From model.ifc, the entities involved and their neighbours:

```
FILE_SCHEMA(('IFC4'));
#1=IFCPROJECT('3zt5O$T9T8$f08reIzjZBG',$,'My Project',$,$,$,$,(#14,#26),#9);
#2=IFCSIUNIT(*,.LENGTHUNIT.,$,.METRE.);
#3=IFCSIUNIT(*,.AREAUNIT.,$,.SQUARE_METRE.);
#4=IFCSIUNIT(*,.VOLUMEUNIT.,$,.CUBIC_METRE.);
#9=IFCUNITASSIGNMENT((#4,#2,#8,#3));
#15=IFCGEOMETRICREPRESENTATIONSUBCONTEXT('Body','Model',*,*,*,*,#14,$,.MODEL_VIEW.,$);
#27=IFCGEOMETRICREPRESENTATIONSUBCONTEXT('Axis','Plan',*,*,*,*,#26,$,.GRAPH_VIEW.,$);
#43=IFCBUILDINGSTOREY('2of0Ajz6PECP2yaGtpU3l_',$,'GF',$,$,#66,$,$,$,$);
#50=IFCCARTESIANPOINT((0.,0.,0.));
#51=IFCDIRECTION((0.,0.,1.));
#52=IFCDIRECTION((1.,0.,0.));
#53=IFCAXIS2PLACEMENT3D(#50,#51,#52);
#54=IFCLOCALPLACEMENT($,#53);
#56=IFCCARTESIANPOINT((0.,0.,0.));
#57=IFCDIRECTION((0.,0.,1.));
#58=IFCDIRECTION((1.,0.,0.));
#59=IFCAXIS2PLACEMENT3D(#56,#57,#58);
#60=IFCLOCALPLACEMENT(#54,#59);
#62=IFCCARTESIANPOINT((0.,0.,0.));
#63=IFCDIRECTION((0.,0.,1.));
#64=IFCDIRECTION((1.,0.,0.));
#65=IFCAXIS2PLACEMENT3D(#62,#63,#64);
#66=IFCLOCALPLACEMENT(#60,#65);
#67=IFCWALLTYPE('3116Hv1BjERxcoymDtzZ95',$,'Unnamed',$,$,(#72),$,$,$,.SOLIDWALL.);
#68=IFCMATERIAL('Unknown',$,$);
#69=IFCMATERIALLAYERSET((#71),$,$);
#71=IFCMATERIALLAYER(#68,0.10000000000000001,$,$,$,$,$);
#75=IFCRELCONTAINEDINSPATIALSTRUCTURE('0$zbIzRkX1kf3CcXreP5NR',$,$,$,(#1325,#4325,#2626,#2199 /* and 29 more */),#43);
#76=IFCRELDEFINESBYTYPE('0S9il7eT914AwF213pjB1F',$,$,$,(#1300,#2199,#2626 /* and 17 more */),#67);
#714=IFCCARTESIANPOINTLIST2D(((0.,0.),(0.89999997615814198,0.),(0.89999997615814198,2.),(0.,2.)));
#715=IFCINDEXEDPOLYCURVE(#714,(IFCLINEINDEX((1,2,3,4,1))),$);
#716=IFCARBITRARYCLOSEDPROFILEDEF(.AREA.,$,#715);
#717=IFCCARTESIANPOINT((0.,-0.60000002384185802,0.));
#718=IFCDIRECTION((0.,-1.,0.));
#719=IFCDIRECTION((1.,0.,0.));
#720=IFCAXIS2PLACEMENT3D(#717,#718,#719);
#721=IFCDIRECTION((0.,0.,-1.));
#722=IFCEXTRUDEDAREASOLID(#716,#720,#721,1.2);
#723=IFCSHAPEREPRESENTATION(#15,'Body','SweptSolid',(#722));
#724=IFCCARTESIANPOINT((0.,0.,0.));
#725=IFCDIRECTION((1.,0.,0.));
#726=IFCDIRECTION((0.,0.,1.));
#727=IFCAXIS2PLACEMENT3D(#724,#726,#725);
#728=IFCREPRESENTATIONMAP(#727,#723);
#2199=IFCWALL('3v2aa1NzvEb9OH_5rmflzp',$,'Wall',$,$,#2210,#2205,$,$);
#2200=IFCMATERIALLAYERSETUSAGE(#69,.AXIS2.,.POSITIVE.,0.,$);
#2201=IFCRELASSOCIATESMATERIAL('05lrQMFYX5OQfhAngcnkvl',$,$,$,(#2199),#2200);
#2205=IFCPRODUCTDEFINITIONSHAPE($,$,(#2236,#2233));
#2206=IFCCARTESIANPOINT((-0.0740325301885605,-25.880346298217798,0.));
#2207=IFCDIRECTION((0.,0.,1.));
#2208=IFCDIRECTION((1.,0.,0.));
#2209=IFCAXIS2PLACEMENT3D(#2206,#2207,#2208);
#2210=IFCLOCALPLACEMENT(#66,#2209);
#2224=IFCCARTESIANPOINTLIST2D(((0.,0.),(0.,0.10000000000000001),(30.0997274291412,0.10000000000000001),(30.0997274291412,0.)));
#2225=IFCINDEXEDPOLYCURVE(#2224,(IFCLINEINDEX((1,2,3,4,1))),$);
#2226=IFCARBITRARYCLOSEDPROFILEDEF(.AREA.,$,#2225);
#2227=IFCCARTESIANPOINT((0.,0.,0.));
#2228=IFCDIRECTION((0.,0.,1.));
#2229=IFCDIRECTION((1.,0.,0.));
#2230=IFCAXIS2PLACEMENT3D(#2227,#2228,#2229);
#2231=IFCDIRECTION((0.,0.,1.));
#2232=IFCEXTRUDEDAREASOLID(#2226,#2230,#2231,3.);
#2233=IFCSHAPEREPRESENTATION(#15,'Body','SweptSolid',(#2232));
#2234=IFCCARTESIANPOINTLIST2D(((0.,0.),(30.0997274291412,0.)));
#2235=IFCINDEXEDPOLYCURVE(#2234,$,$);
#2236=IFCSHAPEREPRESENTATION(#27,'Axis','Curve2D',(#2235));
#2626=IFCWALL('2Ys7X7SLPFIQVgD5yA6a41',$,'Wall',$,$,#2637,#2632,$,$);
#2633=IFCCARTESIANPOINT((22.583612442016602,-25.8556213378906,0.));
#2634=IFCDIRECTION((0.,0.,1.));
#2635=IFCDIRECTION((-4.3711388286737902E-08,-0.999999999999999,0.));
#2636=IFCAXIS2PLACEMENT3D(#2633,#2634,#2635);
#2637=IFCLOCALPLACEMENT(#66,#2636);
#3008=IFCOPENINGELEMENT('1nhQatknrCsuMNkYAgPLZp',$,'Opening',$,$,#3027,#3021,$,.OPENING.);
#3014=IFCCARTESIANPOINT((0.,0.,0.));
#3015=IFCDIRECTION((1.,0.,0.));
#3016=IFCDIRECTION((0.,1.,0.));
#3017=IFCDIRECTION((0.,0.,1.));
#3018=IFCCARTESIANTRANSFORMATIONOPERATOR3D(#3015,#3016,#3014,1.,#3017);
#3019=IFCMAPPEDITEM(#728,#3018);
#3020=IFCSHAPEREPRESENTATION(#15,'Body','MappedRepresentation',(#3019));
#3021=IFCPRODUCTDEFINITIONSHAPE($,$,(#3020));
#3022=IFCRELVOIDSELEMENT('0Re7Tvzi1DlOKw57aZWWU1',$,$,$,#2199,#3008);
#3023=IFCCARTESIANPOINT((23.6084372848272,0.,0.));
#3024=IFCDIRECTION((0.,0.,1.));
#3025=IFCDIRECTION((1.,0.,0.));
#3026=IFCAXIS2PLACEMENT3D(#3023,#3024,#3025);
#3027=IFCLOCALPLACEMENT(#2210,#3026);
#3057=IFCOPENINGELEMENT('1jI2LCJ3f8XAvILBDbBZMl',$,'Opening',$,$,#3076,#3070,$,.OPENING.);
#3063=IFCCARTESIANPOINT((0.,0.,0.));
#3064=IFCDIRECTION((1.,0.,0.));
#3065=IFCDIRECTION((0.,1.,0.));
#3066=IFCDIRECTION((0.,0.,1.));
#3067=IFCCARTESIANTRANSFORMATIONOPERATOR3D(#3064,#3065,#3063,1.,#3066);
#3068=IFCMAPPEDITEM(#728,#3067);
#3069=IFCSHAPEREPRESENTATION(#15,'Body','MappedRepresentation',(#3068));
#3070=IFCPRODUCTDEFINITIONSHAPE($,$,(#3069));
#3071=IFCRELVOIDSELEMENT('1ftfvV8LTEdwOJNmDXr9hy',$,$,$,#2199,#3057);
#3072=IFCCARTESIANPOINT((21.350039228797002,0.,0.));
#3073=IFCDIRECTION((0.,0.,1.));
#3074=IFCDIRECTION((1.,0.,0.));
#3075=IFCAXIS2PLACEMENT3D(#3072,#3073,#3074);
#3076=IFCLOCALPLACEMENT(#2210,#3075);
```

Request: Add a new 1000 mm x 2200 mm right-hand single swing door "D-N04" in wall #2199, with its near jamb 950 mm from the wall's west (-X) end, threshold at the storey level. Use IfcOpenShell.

```python
import numpy as np
import ifcopenshell
import ifcopenshell.api.feature
import ifcopenshell.api.geometry
import ifcopenshell.api.root
import ifcopenshell.api.spatial
import ifcopenshell.geom
import ifcopenshell.util.element
import ifcopenshell.util.placement
import ifcopenshell.util.representation
import ifcopenshell.util.shape
import ifcopenshell.util.unit

model = ifcopenshell.open("model.ifc")
unit_scale = ifcopenshell.util.unit.calculate_unit_scale(model)
settings = ifcopenshell.geom.settings()


def volume(element):
    """Net volume in cubic metres, openings subtracted."""
    shape = ifcopenshell.geom.create_shape(settings, element)
    return ifcopenshell.util.shape.get_volume(shape.geometry)


wall = model.by_guid("3v2aa1NzvEb9OH_5rmflzp")
storey = ifcopenshell.util.element.get_container(wall, ifc_class="IfcBuildingStorey")
context = ifcopenshell.util.representation.get_context(model, "Model", "Body", "MODEL_VIEW")
before = volume(wall)

width, height, from_end, sill = 1, 2.2, 0.95, 0.0  # metres

# The wall runs along its own X axis, and the end named is its -X end.
wall_shape = ifcopenshell.geom.create_shape(settings, wall)
x, y, z = ifcopenshell.util.shape.get_vertices(wall_shape.geometry).T
start = x.min() + from_end
face, thickness = float(y.min()), float(y.max() - y.min())
wall_matrix = ifcopenshell.util.placement.get_local_placement(wall.ObjectPlacement)
level = ifcopenshell.util.placement.get_local_placement(storey.ObjectPlacement)[2, 3]


def in_wall(x, y):
    """Placement at x, y metres in the wall's axes, at sill height."""
    matrix = wall_matrix.copy()
    matrix[:, 3] = wall_matrix @ np.array([x / unit_scale, y / unit_scale, 0.0, 1.0])
    matrix[2, 3] = level + sill / unit_scale
    return matrix


# Opening: a box that overshoots both wall faces by 50 mm.
opening = ifcopenshell.api.root.create_entity(model, ifc_class="IfcOpeningElement", predefined_type="OPENING")
box = ifcopenshell.api.geometry.add_wall_representation(
    model, context=context, length=width, height=height, thickness=thickness + 0.1
)
ifcopenshell.api.geometry.assign_representation(model, product=opening, representation=box)
ifcopenshell.api.geometry.edit_object_placement(model, product=opening, matrix=in_wall(start, face - 0.05), is_si=False)
ifcopenshell.api.feature.add_feature(model, feature=opening, element=wall)

door = ifcopenshell.api.root.create_entity(model, ifc_class="IfcDoor", name="D-N04", predefined_type="DOOR")
door.OverallWidth, door.OverallHeight = width / unit_scale, height / unit_scale
door.OperationType = "SINGLE_SWING_RIGHT"
body = ifcopenshell.api.geometry.add_door_representation(
    model,
    context=context,
    overall_width=door.OverallWidth,
    overall_height=door.OverallHeight,
    operation_type="SINGLE_SWING_RIGHT",
    lining_properties={"LiningDepth": thickness / unit_scale, "ThresholdDepth": thickness / unit_scale},
)
ifcopenshell.api.geometry.assign_representation(model, product=door, representation=body)
ifcopenshell.api.spatial.assign_container(model, products=[door], relating_structure=storey)
ifcopenshell.api.feature.add_filling(model, opening=opening, element=door)

# The lining spans the wall, so the door starts at the wall face.
ifcopenshell.api.geometry.edit_object_placement(model, product=door, matrix=in_wall(start, face), is_si=False)

after = volume(wall)

print(f"wall volume {before:.3f} -> {after:.3f} m3")

model.write("model_updated.ifc")
```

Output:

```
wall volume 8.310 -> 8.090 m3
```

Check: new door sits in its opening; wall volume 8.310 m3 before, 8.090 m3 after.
